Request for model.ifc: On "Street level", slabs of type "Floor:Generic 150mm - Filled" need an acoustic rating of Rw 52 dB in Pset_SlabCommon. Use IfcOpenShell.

First a look at what the model holds.

```python
import ifcopenshell
import ifcopenshell.util.element

model = ifcopenshell.open("model.ifc")
print(model.schema)
storey = next(s for s in model.by_type("IfcBuildingStorey") if s.Name == "Street level")
slabs = [e for e in ifcopenshell.util.element.get_decomposition(storey) if e.is_a("IfcSlab")]
seen = {}
for e in slabs:
    element_type = ifcopenshell.util.element.get_type(e)
    key = (element_type.Name if element_type != e and element_type else None, ifcopenshell.util.element.get_pset(e, "Pset_SlabCommon", "AcousticRating"))
    seen[key] = seen.get(key, 0) + 1
for (name, value), count in sorted(seen.items(), key=str):
    print(count, "x", name, "|", value)
```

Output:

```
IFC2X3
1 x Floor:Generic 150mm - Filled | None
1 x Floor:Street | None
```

```python
import ifcopenshell
import ifcopenshell.api.pset
import ifcopenshell.util.element

model = ifcopenshell.open("model.ifc")

storey = next(s for s in model.by_type("IfcBuildingStorey") if s.Name == "Street level")
slabs = [e for e in ifcopenshell.util.element.get_decomposition(storey) if e.is_a("IfcSlab")]

count = 0
for e in slabs:
    element_type = ifcopenshell.util.element.get_type(e)
    if element_type in (None, e) or element_type.Name != "Floor:Generic 150mm - Filled":
        continue
    # add_pset returns the element's existing set when there is one.
    pset = ifcopenshell.api.pset.add_pset(model, product=e, name="Pset_SlabCommon")
    ifcopenshell.api.pset.edit_pset(model, pset=pset, properties={"AcousticRating": "Rw 52 dB"})
    count += 1

print(count, "slabs updated")

model.write("model_rev.ifc")
```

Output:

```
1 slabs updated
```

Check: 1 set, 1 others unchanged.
